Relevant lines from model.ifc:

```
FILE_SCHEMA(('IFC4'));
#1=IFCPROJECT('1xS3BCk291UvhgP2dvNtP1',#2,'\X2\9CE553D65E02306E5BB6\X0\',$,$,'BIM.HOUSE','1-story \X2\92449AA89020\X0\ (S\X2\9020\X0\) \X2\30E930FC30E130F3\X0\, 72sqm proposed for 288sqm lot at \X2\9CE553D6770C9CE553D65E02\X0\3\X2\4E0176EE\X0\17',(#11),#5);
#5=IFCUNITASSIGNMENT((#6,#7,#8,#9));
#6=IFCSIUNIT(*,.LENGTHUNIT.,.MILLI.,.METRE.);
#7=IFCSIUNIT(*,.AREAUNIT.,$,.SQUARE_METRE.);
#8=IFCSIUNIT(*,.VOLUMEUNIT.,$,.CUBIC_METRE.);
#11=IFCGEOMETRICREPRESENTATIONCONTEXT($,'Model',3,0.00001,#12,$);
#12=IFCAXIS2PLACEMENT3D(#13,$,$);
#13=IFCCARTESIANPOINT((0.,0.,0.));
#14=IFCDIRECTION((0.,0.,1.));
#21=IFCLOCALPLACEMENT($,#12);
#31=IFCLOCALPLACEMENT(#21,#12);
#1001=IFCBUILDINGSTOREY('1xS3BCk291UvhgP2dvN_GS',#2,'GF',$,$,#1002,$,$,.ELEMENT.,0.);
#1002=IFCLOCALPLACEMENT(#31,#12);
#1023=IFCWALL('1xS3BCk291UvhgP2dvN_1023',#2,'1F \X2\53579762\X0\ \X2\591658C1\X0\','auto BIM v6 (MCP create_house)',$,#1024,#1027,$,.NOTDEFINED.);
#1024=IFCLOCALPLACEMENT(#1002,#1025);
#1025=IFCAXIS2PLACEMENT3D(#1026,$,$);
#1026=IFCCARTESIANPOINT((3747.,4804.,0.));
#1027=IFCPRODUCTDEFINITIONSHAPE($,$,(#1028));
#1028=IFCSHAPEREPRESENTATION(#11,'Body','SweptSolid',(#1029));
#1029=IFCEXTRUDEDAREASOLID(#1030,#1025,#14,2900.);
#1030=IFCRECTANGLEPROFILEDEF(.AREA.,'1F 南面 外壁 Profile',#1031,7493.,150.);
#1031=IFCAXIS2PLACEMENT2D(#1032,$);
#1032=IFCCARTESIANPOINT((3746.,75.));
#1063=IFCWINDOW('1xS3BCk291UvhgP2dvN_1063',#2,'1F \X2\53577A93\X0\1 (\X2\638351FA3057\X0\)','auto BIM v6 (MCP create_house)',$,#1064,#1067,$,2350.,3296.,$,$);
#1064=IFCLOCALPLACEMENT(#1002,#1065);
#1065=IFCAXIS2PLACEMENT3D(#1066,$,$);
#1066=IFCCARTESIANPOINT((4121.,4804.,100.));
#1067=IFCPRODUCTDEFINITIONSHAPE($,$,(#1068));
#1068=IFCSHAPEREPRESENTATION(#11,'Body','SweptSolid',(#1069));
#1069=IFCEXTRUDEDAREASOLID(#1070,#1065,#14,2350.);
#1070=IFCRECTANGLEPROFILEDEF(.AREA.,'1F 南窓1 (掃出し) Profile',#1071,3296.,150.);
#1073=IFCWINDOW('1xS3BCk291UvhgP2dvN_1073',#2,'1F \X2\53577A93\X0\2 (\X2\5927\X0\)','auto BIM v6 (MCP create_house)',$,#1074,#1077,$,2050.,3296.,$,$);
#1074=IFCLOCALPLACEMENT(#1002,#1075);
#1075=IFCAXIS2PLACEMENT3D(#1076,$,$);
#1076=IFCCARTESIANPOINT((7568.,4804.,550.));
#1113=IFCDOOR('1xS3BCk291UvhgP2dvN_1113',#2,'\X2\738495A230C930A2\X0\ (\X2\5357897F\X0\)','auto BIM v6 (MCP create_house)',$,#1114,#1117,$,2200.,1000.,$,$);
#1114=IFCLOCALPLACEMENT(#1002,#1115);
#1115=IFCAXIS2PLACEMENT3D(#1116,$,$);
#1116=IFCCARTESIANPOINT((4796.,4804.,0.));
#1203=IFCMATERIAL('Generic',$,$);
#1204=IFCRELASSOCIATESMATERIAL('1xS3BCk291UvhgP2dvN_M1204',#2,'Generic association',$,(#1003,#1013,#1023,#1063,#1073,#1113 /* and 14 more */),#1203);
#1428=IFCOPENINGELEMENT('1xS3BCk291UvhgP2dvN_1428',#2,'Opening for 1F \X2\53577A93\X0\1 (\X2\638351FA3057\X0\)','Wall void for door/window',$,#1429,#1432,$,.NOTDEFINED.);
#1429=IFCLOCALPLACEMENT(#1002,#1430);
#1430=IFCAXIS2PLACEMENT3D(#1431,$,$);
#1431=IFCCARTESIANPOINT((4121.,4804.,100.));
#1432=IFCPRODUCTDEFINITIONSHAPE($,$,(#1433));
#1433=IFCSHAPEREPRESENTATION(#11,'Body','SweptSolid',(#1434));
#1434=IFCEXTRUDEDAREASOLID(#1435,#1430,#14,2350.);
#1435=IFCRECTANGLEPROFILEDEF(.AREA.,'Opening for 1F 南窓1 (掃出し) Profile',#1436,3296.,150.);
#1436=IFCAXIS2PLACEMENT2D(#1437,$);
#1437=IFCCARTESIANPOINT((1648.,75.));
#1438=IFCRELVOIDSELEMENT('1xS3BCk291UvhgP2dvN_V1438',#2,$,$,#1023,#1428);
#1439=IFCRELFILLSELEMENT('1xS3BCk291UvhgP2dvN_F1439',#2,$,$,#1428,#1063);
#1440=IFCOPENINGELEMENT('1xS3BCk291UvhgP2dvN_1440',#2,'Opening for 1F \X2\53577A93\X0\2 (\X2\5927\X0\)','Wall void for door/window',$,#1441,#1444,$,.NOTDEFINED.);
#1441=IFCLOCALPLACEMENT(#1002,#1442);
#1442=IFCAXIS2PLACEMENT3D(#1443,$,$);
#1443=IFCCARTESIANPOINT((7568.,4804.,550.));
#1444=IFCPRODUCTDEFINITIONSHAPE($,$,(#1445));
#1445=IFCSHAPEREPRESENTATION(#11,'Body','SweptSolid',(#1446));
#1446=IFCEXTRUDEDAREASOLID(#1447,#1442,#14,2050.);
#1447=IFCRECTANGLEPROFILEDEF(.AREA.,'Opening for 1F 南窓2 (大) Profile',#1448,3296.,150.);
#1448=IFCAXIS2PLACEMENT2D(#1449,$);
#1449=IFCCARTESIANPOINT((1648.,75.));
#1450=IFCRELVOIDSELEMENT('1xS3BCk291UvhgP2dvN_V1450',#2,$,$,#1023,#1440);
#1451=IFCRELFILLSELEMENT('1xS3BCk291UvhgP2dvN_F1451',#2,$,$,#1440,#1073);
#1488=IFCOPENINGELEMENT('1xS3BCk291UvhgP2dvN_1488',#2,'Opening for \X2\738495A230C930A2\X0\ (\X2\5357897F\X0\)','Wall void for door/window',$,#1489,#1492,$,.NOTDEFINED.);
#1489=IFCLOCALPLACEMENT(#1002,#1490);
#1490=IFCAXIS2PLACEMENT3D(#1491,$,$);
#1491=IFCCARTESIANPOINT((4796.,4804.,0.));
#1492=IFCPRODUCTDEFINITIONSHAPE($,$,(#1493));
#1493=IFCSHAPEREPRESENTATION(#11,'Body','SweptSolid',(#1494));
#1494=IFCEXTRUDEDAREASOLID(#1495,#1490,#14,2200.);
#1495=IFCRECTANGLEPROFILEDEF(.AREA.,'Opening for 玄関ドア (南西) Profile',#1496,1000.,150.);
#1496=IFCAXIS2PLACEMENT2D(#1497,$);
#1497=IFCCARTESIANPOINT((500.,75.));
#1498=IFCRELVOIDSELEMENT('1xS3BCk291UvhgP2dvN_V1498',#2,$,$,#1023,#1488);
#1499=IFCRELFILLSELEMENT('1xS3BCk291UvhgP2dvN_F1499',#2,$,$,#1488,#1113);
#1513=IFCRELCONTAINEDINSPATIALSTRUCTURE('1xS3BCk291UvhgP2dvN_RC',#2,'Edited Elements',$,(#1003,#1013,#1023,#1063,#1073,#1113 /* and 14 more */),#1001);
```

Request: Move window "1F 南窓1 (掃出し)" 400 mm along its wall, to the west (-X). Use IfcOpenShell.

```python
import ifcopenshell
import ifcopenshell.api.geometry
import ifcopenshell.util.placement

model = ifcopenshell.open("model.ifc")

window = model.by_guid("1xS3BCk291UvhgP2dvN_1063")
opening = window.FillsVoids[0].RelatingOpeningElement
wall = opening.VoidsElements[0].RelatingBuildingElement

wall_matrix = ifcopenshell.util.placement.get_local_placement(wall.ObjectPlacement)
shift = wall_matrix[:3, 0] * -400.0
before = ifcopenshell.util.placement.get_local_placement(window.ObjectPlacement)[:3, 3].copy()

# The window is not placed relative to its opening, so move both.
for product in (opening, window):
    matrix = ifcopenshell.util.placement.get_local_placement(product.ObjectPlacement)
    matrix[:3, 3] += shift
    ifcopenshell.api.geometry.edit_object_placement(model, product=product, matrix=matrix, is_si=False)

after = ifcopenshell.util.placement.get_local_placement(window.ObjectPlacement)[:3, 3]
print("window moved by", (after - before).round(3) + 0.0)

model.write("model_edited.ifc")
```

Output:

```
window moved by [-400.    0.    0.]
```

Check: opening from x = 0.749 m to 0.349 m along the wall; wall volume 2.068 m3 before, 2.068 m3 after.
